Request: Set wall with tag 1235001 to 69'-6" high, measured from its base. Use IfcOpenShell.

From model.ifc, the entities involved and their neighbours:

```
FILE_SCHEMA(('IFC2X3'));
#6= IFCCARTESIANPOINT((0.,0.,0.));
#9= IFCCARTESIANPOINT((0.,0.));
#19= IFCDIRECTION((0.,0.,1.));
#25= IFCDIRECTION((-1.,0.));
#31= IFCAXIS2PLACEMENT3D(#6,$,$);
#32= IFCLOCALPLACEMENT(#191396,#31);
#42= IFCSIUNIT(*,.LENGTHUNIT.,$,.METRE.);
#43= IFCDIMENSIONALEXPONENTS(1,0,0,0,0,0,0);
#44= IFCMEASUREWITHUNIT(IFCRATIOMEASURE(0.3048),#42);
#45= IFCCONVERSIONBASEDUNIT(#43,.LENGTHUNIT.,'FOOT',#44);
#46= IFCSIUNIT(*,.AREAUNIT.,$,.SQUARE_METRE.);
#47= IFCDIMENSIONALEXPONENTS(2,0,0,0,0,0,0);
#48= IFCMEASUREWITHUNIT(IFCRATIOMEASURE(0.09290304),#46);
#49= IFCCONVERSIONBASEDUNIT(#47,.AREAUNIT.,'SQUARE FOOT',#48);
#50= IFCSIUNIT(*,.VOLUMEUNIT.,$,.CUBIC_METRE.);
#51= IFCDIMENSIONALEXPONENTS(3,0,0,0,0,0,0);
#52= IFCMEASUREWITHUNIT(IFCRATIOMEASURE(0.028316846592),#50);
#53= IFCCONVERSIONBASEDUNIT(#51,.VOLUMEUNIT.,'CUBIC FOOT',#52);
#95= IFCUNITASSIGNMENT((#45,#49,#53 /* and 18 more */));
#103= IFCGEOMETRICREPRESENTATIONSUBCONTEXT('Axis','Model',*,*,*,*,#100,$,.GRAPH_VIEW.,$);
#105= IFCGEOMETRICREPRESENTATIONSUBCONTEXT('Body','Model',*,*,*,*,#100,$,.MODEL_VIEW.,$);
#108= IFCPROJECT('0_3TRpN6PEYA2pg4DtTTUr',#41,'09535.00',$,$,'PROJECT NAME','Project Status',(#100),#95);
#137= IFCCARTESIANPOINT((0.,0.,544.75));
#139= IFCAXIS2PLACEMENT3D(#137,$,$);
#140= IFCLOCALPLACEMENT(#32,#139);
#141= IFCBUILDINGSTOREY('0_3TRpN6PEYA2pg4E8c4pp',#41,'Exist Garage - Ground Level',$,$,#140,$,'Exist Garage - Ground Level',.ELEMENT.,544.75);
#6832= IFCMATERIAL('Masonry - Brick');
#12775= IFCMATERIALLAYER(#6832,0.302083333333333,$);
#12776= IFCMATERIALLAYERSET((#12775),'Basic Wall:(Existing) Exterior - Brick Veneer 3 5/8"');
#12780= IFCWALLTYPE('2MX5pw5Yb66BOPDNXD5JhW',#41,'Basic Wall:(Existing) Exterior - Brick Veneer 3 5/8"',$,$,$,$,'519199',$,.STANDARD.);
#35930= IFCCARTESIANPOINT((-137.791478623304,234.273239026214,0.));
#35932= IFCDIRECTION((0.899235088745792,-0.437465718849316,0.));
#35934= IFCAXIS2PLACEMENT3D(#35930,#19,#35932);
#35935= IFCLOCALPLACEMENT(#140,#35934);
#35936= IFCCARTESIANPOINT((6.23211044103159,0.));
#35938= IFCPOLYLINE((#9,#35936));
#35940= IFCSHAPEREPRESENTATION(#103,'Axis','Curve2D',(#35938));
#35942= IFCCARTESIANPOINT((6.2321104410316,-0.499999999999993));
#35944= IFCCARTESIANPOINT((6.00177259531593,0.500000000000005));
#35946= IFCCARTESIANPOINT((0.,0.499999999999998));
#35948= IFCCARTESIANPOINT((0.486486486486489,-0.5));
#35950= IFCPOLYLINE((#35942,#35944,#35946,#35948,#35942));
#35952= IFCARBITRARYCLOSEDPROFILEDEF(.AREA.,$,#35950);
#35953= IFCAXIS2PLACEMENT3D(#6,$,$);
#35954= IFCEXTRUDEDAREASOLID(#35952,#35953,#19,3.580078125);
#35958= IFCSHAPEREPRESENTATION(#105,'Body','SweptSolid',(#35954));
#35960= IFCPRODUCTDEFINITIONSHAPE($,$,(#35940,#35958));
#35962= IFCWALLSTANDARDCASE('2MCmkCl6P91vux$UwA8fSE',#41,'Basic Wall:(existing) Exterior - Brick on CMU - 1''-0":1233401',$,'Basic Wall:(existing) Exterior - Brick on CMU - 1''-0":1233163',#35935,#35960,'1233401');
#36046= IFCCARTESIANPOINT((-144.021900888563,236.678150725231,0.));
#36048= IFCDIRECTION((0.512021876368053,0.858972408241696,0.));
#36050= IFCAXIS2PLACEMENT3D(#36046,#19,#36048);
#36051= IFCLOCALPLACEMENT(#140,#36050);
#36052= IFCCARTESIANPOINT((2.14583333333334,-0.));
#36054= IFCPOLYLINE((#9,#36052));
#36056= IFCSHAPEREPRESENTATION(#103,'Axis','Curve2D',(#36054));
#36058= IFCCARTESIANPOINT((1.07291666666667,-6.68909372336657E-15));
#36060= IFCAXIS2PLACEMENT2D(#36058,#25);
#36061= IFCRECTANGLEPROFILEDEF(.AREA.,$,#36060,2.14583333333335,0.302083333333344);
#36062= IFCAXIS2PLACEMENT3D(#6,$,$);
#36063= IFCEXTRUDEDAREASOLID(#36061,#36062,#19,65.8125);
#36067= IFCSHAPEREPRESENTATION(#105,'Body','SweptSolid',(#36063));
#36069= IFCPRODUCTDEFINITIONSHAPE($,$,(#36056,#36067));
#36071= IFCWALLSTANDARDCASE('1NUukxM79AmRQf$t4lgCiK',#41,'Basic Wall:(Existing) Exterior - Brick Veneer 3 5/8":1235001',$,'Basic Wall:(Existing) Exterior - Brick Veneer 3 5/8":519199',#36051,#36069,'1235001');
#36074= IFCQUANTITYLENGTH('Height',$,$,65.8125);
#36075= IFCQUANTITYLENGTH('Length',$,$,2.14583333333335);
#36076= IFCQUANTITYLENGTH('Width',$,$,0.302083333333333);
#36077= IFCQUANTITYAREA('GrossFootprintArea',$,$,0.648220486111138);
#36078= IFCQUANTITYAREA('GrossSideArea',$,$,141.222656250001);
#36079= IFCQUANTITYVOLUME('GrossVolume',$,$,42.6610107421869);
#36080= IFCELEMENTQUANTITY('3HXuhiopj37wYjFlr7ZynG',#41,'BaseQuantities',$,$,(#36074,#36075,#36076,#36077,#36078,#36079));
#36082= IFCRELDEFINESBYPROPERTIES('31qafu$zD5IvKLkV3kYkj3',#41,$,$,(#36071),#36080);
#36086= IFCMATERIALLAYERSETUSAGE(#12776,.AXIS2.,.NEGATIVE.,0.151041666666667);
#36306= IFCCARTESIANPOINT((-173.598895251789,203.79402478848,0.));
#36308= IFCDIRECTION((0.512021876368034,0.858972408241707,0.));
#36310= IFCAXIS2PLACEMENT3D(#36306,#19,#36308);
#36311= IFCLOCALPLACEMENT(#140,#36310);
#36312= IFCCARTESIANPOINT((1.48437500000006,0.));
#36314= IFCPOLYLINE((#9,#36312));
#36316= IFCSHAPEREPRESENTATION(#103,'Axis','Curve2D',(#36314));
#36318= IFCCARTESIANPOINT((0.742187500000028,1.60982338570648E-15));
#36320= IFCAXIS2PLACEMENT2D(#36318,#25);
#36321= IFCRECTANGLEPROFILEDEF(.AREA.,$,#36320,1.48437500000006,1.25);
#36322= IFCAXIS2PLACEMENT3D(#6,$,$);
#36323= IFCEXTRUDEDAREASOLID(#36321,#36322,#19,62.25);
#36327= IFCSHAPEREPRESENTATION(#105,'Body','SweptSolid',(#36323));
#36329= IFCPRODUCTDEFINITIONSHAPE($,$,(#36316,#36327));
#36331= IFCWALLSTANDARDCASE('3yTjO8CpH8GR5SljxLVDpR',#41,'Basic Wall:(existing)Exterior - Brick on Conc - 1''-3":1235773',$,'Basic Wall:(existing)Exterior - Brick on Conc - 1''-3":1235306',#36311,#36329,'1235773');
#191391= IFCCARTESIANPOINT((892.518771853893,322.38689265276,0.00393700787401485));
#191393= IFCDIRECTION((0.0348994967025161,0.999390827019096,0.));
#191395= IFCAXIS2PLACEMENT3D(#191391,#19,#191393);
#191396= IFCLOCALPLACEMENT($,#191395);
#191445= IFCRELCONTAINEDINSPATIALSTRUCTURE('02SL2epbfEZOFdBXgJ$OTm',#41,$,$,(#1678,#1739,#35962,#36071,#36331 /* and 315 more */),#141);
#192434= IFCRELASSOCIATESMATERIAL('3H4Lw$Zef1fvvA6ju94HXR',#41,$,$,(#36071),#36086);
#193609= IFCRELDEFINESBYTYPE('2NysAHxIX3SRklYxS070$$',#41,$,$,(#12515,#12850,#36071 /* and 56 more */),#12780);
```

```python
import ifcopenshell
import ifcopenshell.api.pset
import ifcopenshell.geom
import ifcopenshell.util.element
import ifcopenshell.util.representation
import ifcopenshell.util.shape
import ifcopenshell.util.unit

model = ifcopenshell.open("model.ifc")
unit_scale = ifcopenshell.util.unit.calculate_unit_scale(model)
area_scale = ifcopenshell.util.unit.calculate_unit_scale(model, "AREAUNIT")
volume_scale = ifcopenshell.util.unit.calculate_unit_scale(model, "VOLUMEUNIT")
settings = ifcopenshell.geom.settings()


def volume(element):
    """Net volume in cubic metres, openings subtracted."""
    shape = ifcopenshell.geom.create_shape(settings, element)
    return ifcopenshell.util.shape.get_volume(shape.geometry)


wall = model.by_id(36071)
before = volume(wall)

body = ifcopenshell.util.representation.get_representation(wall, "Model", "Body")
solid = body.Items[0]
old_height = solid.Depth
solid.Depth = 834 * 0.0254 / unit_scale
after = volume(wall)

# Update the stored height, areas and volumes.
qto = model.by_id(ifcopenshell.util.element.get_pset(wall, "BaseQuantities", should_inherit=False)["id"])
ifcopenshell.api.pset.edit_qto(model, qto=qto, properties={
    "Height": solid.Depth,
    "GrossSideArea": ifcopenshell.util.element.get_pset(wall, "BaseQuantities", "GrossSideArea") * solid.Depth / old_height,
    "GrossVolume": ifcopenshell.util.element.get_pset(wall, "BaseQuantities", "GrossVolume") * solid.Depth / old_height,
})

print(f"height {old_height:g} -> {solid.Depth:g}, volume {before:.3f} -> {after:.3f} m3")

model.write("model_updated.ifc")
```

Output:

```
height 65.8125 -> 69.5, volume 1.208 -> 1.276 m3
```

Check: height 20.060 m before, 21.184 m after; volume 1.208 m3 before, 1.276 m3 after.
